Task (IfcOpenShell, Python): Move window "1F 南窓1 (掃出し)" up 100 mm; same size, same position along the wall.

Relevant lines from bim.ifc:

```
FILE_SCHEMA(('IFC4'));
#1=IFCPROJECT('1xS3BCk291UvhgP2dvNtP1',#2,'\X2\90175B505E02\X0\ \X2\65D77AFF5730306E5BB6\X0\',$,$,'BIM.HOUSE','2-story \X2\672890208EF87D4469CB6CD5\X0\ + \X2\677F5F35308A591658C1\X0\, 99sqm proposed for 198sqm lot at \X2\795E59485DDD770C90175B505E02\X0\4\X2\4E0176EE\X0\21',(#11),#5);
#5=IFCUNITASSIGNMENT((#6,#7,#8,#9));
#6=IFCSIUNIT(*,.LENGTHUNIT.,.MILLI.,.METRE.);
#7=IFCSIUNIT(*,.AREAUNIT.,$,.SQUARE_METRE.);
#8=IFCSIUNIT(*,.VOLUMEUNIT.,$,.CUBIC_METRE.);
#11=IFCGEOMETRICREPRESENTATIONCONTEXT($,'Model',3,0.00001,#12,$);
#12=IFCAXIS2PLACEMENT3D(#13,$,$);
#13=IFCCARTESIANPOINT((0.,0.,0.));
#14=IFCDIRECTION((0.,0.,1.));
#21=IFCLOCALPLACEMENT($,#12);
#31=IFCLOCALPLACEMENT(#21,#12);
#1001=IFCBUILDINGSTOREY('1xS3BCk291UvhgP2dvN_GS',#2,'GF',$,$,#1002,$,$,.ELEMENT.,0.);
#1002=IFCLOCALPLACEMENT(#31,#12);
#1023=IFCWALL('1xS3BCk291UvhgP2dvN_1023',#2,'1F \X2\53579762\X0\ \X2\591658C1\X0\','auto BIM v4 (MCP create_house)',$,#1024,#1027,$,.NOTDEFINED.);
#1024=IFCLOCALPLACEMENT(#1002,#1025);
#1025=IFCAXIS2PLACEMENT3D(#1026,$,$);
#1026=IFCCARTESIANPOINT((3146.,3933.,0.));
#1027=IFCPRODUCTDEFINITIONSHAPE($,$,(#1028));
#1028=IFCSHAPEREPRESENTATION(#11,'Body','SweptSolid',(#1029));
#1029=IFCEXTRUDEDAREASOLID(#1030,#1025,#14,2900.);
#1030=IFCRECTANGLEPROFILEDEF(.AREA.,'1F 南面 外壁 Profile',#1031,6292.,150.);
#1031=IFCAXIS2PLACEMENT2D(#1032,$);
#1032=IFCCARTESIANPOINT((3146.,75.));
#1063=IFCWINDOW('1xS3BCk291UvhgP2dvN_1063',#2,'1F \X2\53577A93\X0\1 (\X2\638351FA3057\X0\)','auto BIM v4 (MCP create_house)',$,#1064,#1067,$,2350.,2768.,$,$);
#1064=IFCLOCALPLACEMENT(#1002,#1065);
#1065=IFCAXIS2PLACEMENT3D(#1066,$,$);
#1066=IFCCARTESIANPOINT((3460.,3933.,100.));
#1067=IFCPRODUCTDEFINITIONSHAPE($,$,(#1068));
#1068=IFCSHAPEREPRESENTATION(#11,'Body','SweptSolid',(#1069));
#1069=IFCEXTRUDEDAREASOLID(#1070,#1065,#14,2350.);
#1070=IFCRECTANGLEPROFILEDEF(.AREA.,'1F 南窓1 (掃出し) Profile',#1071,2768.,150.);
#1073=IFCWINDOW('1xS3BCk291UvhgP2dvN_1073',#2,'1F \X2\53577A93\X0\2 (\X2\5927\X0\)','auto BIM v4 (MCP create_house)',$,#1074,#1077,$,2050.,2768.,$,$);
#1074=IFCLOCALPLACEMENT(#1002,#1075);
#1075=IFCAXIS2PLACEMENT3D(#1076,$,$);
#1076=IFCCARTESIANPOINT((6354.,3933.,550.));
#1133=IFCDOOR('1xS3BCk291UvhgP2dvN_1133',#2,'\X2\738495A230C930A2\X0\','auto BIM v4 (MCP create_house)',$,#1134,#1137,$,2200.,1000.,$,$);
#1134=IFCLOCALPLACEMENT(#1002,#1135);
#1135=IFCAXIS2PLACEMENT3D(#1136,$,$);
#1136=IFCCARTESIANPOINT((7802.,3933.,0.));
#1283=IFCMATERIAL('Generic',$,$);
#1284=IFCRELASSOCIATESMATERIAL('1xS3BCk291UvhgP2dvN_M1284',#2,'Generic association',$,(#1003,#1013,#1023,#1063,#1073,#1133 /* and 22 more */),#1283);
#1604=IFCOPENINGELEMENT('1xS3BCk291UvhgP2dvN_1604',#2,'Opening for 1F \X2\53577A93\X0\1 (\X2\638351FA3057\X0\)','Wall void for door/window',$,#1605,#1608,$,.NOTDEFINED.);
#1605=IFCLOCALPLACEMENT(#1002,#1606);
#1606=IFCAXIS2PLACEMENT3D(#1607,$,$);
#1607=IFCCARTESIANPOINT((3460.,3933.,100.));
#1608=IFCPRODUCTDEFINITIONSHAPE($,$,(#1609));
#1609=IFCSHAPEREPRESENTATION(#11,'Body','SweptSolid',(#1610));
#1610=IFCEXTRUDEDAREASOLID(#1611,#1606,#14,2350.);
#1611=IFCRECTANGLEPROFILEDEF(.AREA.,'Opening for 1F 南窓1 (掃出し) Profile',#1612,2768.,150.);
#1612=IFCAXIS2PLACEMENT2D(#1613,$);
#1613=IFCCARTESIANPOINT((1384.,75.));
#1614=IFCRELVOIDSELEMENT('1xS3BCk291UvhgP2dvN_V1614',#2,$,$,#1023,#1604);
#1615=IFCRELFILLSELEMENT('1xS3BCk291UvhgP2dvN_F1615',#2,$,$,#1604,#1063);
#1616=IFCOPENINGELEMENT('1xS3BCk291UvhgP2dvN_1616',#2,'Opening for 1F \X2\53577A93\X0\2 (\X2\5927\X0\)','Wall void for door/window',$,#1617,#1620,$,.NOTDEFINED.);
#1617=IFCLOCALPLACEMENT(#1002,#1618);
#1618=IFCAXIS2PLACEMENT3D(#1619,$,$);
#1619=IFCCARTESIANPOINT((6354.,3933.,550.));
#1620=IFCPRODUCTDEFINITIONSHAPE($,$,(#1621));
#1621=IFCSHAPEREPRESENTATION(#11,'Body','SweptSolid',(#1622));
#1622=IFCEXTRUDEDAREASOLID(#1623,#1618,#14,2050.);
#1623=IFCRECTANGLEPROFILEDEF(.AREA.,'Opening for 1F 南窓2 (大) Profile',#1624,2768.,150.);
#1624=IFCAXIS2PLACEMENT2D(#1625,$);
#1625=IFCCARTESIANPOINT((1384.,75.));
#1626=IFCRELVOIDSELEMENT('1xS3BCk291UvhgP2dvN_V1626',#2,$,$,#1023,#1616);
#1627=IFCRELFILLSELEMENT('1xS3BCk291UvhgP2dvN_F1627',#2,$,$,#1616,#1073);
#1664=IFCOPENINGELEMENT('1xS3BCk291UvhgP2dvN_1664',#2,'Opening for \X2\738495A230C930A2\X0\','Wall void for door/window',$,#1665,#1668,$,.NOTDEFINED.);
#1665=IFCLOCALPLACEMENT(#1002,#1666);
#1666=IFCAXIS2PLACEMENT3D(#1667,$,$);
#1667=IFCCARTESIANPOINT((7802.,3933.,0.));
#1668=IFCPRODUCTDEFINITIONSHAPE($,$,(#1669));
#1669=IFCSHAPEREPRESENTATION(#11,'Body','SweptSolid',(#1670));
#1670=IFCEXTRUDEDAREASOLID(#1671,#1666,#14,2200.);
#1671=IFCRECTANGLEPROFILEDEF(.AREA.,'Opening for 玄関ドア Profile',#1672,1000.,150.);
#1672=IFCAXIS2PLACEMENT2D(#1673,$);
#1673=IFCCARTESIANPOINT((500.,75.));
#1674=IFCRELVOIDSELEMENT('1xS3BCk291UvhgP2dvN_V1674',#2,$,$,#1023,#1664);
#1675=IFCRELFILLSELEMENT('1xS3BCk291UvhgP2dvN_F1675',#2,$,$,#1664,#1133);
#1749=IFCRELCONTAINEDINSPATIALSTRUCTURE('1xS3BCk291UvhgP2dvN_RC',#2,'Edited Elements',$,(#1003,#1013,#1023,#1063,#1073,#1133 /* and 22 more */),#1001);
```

```python
import numpy as np
import ifcopenshell
import ifcopenshell.api.geometry
import ifcopenshell.util.placement
import ifcopenshell.util.unit

model = ifcopenshell.open("bim.ifc")
unit_scale = ifcopenshell.util.unit.calculate_unit_scale(model)

window = model.by_guid("1xS3BCk291UvhgP2dvN_1063")
opening = window.FillsVoids[0].RelatingOpeningElement
dz = 0.1 / unit_scale

shift = np.array([0.0, 0.0, dz])
# The window is not placed relative to its opening, so move both.
for product in (opening, window):
    matrix = ifcopenshell.util.placement.get_local_placement(product.ObjectPlacement)
    matrix[:3, 3] += shift
    ifcopenshell.api.geometry.edit_object_placement(model, product=product, matrix=matrix, is_si=False)

print(f"moved by {dz * unit_scale:+.3f} m")

model.write("bim-out.ifc")
```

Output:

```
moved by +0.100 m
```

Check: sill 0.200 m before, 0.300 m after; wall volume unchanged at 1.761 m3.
